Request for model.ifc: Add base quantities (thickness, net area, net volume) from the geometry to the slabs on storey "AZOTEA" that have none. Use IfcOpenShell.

First a look at what the model holds.

```python
import ifcopenshell
import ifcopenshell.util.element
import ifcopenshell.util.unit

model = ifcopenshell.open("model.ifc")
print(model.schema)
for unit_type in ("LENGTHUNIT", "AREAUNIT", "VOLUMEUNIT"):
    print(unit_type, ifcopenshell.util.unit.calculate_unit_scale(model, unit_type))
storey = next(s for s in model.by_type("IfcBuildingStorey") if s.Name == "AZOTEA")
slabs = [e for e in ifcopenshell.util.element.get_decomposition(storey) if e.is_a("IfcSlab")]
for e in sorted(slabs, key=lambda e: e.id()):
    print(e.id(), e.is_a(), e.Name, list(ifcopenshell.util.element.get_psets(e, qtos_only=True)), sep=" | ")
```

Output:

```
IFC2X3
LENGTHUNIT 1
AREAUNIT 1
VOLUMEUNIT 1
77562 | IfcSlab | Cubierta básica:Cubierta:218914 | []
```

```python
import ifcopenshell
import ifcopenshell.api.pset
import ifcopenshell.geom
import ifcopenshell.util.element
import ifcopenshell.util.shape
import ifcopenshell.util.unit

model = ifcopenshell.open("model.ifc")
unit_scale = ifcopenshell.util.unit.calculate_unit_scale(model)
area_scale = ifcopenshell.util.unit.calculate_unit_scale(model, "AREAUNIT")
volume_scale = ifcopenshell.util.unit.calculate_unit_scale(model, "VOLUMEUNIT")
settings = ifcopenshell.geom.settings()

storey = next(s for s in model.by_type("IfcBuildingStorey") if s.Name == "AZOTEA")
slabs = [e for e in ifcopenshell.util.element.get_decomposition(storey) if e.is_a("IfcSlab")]

for e in sorted(slabs, key=lambda e: e.id()):
    if ifcopenshell.util.element.get_psets(e, qtos_only=True, should_inherit=False):
        continue
    # Geometry comes back in metres, in the element's own axes.
    shape = ifcopenshell.geom.create_shape(settings, e)
    values = {
        "Width": ifcopenshell.util.shape.get_z(shape.geometry) / unit_scale,
        "NetArea": ifcopenshell.util.shape.get_footprint_area(shape.geometry) / area_scale,
        "NetVolume": ifcopenshell.util.shape.get_volume(shape.geometry) / volume_scale,
    }
    qto = ifcopenshell.api.pset.add_qto(model, product=e, name="BaseQuantities")
    ifcopenshell.api.pset.edit_qto(model, qto=qto, properties=values)
    print(e.id(), {k: round(v, 3) for k, v in values.items()})

model.write("model_rev.ifc")
```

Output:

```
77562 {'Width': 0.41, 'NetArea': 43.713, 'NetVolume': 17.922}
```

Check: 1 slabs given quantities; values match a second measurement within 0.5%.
